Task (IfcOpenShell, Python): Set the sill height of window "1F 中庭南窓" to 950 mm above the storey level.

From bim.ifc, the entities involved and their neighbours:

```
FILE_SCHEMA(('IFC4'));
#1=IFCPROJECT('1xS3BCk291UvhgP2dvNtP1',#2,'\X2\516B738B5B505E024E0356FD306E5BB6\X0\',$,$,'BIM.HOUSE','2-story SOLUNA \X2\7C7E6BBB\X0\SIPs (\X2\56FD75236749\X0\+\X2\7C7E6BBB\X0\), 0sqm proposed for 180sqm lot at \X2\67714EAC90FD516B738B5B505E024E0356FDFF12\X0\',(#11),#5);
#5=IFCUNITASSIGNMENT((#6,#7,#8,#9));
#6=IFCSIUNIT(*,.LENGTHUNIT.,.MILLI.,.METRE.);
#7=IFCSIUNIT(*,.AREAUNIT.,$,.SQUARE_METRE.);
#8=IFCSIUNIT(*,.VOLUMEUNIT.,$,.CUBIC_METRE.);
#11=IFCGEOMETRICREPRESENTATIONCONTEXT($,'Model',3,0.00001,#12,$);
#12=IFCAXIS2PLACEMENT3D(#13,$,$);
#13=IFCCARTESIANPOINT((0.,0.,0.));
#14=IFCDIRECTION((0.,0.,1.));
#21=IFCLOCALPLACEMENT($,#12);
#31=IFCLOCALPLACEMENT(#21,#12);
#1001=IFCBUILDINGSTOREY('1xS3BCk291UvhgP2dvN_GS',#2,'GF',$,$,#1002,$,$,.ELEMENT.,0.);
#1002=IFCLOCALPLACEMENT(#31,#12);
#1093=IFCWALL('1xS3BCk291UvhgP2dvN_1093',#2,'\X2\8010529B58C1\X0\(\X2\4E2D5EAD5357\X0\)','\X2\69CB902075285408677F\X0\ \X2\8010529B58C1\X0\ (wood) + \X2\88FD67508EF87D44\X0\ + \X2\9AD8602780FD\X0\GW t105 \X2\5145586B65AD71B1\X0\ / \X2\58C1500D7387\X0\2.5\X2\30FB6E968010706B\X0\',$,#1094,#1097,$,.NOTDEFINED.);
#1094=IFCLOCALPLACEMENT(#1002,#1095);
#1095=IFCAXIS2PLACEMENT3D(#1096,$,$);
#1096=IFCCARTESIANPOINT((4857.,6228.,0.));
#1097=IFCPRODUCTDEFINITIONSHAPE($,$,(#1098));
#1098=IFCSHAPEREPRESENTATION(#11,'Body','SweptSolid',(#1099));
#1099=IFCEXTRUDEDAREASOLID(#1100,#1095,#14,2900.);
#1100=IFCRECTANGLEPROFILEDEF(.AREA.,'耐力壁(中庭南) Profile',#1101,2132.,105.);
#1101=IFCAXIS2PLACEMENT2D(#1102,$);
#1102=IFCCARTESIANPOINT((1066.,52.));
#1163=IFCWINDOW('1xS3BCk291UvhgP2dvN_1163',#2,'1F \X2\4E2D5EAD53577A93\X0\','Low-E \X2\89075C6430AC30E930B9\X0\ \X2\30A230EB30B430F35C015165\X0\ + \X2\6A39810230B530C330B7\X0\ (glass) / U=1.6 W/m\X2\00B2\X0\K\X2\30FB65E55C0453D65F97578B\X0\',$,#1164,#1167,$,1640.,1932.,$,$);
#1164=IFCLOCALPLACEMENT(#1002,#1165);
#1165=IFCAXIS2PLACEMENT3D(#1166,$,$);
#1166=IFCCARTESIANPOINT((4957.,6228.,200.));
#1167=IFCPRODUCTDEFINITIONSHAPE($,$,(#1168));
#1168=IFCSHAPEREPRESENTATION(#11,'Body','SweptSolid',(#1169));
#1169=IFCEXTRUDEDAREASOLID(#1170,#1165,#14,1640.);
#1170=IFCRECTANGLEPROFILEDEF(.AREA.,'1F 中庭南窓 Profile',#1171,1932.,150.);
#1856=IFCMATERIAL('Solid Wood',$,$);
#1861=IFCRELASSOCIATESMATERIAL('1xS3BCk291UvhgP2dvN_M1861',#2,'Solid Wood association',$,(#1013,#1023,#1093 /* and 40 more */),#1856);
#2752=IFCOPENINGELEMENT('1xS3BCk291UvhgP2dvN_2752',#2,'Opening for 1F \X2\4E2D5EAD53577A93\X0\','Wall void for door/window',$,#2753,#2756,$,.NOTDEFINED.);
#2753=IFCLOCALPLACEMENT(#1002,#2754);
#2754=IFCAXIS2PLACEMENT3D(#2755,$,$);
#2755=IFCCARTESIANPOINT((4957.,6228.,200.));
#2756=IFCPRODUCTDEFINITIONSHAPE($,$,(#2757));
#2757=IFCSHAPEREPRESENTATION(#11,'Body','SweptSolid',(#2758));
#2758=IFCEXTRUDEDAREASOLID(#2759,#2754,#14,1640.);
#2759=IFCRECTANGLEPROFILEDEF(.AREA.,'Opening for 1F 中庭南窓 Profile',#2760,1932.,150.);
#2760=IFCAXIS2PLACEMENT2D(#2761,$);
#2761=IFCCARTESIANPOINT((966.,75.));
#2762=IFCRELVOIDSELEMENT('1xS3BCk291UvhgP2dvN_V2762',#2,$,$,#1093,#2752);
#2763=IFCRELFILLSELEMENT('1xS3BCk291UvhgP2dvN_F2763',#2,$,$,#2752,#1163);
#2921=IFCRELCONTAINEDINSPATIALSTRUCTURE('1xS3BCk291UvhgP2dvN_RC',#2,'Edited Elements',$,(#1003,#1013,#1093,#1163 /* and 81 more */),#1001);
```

```python
import numpy as np
import ifcopenshell
import ifcopenshell.api.geometry
import ifcopenshell.geom
import ifcopenshell.util.element
import ifcopenshell.util.placement
import ifcopenshell.util.shape
import ifcopenshell.util.unit

model = ifcopenshell.open("bim.ifc")
unit_scale = ifcopenshell.util.unit.calculate_unit_scale(model)

window = model.by_id(1163)
opening = window.FillsVoids[0].RelatingOpeningElement
storey = ifcopenshell.util.element.get_container(window, ifc_class="IfcBuildingStorey")
level = ifcopenshell.util.placement.get_local_placement(storey.ObjectPlacement)[2, 3]

# The opening's origin need not be at the sill, so measure its lowest point.
shape = ifcopenshell.geom.create_shape(ifcopenshell.geom.settings(), opening)
bottom = ifcopenshell.util.shape.get_shape_bottom_elevation(shape, shape.geometry) / unit_scale
dz = level + 950.0 - bottom

shift = np.array([0.0, 0.0, dz])
# The window is not placed relative to its opening, so move both.
for product in (opening, window):
    matrix = ifcopenshell.util.placement.get_local_placement(product.ObjectPlacement)
    matrix[:3, 3] += shift
    ifcopenshell.api.geometry.edit_object_placement(model, product=product, matrix=matrix, is_si=False)

print(f"moved by {dz * unit_scale:+.3f} m")

model.write("bim-out.ifc")
```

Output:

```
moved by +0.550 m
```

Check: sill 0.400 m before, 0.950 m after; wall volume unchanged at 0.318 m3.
